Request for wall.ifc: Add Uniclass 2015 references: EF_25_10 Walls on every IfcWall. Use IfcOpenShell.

First a look at what the model holds.

```python
import ifcopenshell

model = ifcopenshell.open("wall.ifc")
print(model.schema)
print("classifications:", [c.Name for c in model.by_type("IfcClassification")])
for ifc_class in ("IfcDoor", "IfcRoof", "IfcStair", "IfcWall", "IfcWindow"):
    print(ifc_class, len(model.by_type(ifc_class)))
```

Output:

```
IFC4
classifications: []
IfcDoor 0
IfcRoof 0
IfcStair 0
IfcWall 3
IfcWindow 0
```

```python
import ifcopenshell
import ifcopenshell.api.classification

model = ifcopenshell.open("wall.ifc")

system = ifcopenshell.api.classification.add_classification(model, classification="Uniclass 2015")

codes = {
    "IfcWall": ("EF_25_10", "Walls"),
}
for ifc_class, (code, name) in codes.items():
    products = model.by_type(ifc_class)
    ifcopenshell.api.classification.add_reference(
        model, products=products, classification=system, identification=code, name=name
    )
    print(code, len(products))

model.write("wall_edited.ifc")
```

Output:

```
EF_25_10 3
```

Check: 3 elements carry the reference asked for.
